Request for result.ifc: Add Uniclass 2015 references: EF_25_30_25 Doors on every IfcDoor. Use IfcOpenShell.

First a look at what the model holds.

```python
import ifcopenshell

model = ifcopenshell.open("result.ifc")
print(model.schema)
print("classifications:", [c.Name for c in model.by_type("IfcClassification")])
for ifc_class in ("IfcDoor", "IfcRoof", "IfcStair", "IfcWall", "IfcWindow"):
    print(ifc_class, len(model.by_type(ifc_class)))
```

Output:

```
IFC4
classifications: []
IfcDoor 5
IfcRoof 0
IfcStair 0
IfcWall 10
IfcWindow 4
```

```python
import ifcopenshell
import ifcopenshell.api.classification

model = ifcopenshell.open("result.ifc")

system = ifcopenshell.api.classification.add_classification(model, classification="Uniclass 2015")

codes = {
    "IfcDoor": ("EF_25_30_25", "Doors"),
}
for ifc_class, (code, name) in codes.items():
    products = model.by_type(ifc_class)
    ifcopenshell.api.classification.add_reference(
        model, products=products, classification=system, identification=code, name=name
    )
    print(code, len(products))

model.write("result_v2.ifc")
```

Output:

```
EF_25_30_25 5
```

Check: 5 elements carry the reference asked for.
